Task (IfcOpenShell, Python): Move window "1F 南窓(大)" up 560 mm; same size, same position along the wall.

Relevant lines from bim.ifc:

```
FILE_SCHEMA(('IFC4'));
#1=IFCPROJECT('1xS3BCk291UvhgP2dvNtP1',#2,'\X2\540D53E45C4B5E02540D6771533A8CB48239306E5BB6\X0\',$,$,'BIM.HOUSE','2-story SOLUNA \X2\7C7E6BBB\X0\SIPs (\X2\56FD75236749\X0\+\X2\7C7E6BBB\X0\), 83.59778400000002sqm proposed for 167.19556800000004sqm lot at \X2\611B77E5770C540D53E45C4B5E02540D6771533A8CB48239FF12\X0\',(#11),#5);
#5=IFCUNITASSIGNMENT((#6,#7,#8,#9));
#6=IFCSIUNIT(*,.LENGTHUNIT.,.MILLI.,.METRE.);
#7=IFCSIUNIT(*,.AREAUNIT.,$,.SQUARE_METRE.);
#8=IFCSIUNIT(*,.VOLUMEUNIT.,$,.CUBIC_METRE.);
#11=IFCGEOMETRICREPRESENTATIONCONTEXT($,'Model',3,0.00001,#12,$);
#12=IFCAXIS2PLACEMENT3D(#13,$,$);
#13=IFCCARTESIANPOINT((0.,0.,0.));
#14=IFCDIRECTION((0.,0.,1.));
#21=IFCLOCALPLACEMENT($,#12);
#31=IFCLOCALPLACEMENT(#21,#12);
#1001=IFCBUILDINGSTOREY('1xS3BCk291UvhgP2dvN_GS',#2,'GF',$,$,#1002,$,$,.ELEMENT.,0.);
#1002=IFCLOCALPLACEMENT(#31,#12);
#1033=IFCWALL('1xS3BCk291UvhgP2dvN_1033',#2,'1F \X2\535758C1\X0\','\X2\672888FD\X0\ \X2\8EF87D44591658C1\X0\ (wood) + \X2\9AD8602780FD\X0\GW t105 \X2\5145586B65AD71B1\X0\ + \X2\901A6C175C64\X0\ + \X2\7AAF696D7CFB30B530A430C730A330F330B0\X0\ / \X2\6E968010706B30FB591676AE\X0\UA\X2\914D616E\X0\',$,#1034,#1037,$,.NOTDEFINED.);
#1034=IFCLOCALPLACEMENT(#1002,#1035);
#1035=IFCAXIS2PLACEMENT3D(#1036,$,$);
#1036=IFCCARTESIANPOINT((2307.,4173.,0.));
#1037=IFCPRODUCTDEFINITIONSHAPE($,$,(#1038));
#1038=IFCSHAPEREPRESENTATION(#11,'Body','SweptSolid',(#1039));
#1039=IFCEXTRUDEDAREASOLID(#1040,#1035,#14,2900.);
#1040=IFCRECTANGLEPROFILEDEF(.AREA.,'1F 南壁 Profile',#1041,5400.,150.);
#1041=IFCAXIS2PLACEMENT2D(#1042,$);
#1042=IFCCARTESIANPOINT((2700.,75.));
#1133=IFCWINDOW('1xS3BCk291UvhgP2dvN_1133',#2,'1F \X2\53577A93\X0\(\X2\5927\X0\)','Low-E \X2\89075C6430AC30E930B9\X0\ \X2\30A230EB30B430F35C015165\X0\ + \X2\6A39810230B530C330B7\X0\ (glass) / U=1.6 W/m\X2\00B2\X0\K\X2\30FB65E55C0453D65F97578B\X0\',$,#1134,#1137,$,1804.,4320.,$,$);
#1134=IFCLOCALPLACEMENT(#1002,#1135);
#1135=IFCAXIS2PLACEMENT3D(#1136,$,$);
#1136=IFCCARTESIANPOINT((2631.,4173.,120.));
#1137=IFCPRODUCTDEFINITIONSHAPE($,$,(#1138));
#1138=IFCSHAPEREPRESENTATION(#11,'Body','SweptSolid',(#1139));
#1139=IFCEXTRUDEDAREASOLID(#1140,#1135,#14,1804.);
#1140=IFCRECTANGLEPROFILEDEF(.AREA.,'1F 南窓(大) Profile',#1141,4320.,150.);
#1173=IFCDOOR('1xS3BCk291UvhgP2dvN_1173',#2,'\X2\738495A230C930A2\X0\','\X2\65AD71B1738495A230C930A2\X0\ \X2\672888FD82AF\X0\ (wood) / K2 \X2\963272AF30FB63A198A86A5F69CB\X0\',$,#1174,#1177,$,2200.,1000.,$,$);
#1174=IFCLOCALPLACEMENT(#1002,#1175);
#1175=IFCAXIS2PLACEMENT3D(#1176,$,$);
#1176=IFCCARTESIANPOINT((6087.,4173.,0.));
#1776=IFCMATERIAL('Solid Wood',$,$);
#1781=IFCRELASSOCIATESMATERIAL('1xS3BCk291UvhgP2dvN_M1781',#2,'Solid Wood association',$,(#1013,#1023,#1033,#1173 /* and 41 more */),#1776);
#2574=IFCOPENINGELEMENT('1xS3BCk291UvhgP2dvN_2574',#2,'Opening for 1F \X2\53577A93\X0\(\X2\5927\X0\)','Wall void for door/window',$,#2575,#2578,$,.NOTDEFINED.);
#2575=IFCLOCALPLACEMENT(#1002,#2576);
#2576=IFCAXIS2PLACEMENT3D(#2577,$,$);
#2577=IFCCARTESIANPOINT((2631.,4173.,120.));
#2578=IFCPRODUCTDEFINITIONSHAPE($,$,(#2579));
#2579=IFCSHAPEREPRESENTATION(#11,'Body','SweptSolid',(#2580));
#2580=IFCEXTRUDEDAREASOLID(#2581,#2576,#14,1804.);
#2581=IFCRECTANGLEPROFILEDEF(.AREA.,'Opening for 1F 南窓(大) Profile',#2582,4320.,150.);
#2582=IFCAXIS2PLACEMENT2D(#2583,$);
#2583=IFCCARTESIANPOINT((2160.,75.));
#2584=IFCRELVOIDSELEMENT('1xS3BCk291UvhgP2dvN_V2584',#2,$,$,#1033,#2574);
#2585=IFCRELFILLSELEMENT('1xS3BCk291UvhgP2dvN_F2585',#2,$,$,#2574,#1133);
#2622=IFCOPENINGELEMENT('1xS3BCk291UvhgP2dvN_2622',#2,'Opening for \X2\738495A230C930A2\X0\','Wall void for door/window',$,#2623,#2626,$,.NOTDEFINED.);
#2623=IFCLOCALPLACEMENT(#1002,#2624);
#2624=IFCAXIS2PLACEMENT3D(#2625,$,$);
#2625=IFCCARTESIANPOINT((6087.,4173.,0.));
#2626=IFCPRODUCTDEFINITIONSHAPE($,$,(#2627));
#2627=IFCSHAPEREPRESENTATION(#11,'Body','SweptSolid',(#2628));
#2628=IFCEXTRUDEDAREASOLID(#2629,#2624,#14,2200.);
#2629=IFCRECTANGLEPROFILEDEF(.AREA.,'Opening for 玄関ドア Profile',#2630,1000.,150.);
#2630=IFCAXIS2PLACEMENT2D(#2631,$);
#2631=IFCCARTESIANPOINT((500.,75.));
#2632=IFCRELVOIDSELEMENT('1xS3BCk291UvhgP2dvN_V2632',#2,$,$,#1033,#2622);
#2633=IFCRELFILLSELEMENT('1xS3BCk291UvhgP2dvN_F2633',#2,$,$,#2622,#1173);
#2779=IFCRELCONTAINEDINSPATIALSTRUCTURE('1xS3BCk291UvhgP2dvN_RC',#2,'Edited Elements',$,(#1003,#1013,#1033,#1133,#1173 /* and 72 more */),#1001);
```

```python
import numpy as np
import ifcopenshell
import ifcopenshell.api.geometry
import ifcopenshell.util.placement
import ifcopenshell.util.unit

model = ifcopenshell.open("bim.ifc")
unit_scale = ifcopenshell.util.unit.calculate_unit_scale(model)

window = model.by_guid("1xS3BCk291UvhgP2dvN_1133")
opening = window.FillsVoids[0].RelatingOpeningElement
dz = 560.0

shift = np.array([0.0, 0.0, dz])
# The window is not placed relative to its opening, so move both.
for product in (opening, window):
    matrix = ifcopenshell.util.placement.get_local_placement(product.ObjectPlacement)
    matrix[:3, 3] += shift
    ifcopenshell.api.geometry.edit_object_placement(model, product=product, matrix=matrix, is_si=False)

print(f"moved by {dz * unit_scale:+.3f} m")

model.write("bim-out.ifc")
```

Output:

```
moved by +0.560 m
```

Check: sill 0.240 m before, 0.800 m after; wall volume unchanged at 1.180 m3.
